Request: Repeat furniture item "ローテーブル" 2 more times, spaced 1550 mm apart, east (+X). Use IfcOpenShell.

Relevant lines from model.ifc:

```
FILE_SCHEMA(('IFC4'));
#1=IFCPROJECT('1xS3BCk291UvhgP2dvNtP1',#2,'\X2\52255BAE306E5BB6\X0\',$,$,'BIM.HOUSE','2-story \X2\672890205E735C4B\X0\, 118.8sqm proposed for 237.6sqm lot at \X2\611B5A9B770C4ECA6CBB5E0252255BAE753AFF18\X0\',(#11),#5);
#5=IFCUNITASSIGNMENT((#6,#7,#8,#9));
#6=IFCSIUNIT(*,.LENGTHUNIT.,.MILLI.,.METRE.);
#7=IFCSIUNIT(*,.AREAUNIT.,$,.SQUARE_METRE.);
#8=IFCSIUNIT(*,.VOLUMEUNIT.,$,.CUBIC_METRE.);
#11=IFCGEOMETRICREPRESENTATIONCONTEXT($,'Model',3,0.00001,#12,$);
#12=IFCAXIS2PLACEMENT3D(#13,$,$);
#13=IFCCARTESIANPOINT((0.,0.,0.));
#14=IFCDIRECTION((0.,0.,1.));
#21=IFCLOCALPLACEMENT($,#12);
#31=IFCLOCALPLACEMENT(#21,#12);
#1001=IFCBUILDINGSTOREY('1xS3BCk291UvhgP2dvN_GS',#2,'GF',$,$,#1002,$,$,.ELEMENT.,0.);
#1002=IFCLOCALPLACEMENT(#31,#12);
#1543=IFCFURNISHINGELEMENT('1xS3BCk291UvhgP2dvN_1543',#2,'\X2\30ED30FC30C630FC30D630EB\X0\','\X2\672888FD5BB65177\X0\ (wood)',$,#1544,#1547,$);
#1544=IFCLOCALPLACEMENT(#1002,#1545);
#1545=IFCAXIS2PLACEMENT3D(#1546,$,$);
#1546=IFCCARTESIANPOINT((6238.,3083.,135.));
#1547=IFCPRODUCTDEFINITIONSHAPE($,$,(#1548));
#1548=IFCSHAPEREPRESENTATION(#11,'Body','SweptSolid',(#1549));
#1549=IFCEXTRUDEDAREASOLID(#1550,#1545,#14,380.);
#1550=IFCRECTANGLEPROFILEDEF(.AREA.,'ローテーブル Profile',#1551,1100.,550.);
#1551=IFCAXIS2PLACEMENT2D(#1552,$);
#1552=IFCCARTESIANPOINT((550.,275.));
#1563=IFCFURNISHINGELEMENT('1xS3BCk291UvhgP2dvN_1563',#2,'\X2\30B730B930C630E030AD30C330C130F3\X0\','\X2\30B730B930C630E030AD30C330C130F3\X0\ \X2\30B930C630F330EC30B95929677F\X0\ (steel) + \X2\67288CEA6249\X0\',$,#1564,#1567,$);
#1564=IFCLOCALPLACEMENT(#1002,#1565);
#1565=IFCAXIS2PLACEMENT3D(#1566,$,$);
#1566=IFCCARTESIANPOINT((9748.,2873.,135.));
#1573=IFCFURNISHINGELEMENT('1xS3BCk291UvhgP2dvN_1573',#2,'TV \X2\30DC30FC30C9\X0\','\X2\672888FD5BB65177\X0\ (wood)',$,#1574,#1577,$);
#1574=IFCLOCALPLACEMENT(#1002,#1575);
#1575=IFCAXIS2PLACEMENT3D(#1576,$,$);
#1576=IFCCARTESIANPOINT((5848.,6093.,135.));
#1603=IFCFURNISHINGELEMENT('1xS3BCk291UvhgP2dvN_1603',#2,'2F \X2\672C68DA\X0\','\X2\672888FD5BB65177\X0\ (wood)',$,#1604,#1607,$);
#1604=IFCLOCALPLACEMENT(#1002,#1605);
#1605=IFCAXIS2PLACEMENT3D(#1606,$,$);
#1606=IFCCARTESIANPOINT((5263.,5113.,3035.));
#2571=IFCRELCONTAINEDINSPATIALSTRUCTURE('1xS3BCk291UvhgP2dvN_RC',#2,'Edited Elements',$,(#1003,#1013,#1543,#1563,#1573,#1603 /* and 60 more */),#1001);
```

```python
import numpy as np
import ifcopenshell
import ifcopenshell.api.geometry
import ifcopenshell.api.root
import ifcopenshell.util.element
import ifcopenshell.util.placement
import ifcopenshell.util.unit

model = ifcopenshell.open("model.ifc")
unit_scale = ifcopenshell.util.unit.calculate_unit_scale(model)


def reuse_history(source, copy):
    """copy_class also copies each property set's owner history, people and application; keep the originals."""
    for rel in copy.IsDefinedBy:
        if rel.is_a("IfcRelDefinesByProperties") and (history := rel.RelatingPropertyDefinition.OwnerHistory):
            rel.RelatingPropertyDefinition.OwnerHistory = source.OwnerHistory
            ifcopenshell.util.element.remove_deep2(model, history)


source = model.by_guid("1xS3BCk291UvhgP2dvN_1543")
base = ifcopenshell.util.placement.get_local_placement(source.ObjectPlacement)
step = np.array([1.0, 0.0, 0.0]) * 1.55 / unit_scale

for i in range(1, 3):
    copy = ifcopenshell.api.root.copy_class(model, product=source)
    copy.Representation = ifcopenshell.util.element.copy_deep(
        model, source.Representation, exclude=["IfcGeometricRepresentationContext", "IfcRepresentationMap"]
    )
    reuse_history(source, copy)
    matrix = base.copy()
    matrix[:3, 3] += i * step
    print("added at", matrix[:3, 3].round(3) + 0.0)
    ifcopenshell.api.geometry.edit_object_placement(model, product=copy, matrix=matrix, is_si=False)

model.write("model-out.ifc")
```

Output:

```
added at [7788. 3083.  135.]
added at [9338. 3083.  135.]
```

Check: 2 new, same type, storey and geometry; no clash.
